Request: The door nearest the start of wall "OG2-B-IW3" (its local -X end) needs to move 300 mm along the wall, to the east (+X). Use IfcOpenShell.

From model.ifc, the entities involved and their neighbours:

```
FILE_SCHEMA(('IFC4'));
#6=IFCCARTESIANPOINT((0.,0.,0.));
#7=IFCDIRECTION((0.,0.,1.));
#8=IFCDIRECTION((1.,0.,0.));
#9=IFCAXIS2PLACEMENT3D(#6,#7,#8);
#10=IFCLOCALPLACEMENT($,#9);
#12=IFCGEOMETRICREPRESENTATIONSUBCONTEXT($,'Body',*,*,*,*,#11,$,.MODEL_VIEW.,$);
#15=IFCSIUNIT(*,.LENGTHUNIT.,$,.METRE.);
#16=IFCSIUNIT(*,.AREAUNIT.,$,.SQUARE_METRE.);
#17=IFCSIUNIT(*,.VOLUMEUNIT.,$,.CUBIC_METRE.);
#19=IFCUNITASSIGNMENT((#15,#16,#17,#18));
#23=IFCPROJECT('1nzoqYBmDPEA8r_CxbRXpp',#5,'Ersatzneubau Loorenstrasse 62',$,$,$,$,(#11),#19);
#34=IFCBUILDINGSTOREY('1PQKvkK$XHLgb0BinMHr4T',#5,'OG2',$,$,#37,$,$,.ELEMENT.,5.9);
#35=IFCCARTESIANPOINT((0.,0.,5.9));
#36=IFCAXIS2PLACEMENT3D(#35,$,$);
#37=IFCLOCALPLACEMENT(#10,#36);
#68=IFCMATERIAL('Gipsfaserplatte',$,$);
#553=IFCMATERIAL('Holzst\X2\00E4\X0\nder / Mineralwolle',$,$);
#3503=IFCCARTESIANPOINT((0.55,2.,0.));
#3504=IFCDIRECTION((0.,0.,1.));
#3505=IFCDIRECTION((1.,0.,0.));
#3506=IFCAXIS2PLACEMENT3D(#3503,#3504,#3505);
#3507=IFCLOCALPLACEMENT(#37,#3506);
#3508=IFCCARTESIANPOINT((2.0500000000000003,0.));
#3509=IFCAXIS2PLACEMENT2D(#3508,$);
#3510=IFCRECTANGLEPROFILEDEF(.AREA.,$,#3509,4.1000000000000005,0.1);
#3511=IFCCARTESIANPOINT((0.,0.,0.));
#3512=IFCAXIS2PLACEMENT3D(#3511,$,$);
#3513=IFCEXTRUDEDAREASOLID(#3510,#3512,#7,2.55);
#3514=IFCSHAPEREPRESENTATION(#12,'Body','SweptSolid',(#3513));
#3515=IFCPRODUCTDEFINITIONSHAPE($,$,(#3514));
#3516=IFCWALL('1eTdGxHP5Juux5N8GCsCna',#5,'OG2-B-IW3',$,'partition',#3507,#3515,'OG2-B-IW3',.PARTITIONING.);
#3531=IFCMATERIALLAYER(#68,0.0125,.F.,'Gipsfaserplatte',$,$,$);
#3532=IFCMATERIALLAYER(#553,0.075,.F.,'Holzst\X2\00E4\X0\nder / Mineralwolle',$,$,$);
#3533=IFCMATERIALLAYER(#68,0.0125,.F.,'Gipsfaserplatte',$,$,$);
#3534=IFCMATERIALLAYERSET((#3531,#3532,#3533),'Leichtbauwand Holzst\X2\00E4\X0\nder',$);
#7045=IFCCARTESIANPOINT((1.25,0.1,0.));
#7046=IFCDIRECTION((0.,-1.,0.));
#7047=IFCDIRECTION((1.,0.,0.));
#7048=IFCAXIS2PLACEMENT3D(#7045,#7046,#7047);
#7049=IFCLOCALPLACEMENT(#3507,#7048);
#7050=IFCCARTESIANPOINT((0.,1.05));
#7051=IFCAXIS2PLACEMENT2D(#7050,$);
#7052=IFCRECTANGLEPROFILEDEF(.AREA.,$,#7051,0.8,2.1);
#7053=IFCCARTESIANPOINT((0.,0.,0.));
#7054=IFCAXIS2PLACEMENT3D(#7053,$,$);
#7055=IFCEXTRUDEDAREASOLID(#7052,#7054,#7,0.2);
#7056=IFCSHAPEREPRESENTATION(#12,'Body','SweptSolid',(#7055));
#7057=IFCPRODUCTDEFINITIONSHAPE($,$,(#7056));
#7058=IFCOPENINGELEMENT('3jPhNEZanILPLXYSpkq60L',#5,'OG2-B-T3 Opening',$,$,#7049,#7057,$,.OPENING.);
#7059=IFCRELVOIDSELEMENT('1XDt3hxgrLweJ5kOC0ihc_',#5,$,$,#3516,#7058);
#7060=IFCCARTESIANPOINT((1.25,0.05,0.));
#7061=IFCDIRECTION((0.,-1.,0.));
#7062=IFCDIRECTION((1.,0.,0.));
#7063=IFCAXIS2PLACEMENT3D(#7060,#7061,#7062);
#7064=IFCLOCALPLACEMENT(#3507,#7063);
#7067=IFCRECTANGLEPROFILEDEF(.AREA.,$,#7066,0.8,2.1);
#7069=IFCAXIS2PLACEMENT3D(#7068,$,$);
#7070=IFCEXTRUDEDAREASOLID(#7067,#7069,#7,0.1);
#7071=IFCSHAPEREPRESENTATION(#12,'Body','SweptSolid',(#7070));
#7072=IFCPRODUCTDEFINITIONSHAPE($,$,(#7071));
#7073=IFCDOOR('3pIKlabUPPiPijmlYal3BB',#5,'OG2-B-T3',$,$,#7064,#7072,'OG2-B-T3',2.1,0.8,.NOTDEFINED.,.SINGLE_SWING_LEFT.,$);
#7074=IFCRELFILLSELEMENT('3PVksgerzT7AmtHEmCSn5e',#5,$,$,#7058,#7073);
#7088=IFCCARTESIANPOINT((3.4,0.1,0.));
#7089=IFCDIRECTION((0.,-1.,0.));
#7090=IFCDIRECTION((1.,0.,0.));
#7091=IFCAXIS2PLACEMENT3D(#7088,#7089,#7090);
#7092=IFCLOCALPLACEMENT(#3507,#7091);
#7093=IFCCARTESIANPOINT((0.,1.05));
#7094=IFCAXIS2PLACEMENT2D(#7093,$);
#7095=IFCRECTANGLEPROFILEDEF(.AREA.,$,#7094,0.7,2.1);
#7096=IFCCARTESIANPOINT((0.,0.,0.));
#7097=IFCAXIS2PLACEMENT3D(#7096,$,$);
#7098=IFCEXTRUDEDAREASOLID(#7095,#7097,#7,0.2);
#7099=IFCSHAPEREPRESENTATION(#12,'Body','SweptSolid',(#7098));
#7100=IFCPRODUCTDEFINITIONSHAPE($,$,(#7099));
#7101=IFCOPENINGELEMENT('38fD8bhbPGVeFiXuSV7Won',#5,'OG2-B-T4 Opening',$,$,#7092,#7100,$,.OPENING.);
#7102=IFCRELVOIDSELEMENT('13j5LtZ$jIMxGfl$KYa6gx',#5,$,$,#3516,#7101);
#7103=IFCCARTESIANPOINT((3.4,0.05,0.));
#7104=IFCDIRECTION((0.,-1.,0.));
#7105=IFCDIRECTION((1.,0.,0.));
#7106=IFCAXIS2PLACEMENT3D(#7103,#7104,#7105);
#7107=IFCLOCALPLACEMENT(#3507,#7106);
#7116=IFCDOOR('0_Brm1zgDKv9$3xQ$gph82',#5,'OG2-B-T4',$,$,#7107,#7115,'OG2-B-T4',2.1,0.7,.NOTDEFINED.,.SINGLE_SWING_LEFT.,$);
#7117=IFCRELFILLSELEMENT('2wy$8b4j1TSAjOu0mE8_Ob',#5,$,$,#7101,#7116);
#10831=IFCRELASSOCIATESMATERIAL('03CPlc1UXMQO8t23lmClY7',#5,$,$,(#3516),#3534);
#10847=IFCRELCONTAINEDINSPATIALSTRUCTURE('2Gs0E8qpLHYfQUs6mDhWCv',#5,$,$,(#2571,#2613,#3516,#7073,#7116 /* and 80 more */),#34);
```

```python
import ifcopenshell
import ifcopenshell.api.geometry
import ifcopenshell.util.placement

model = ifcopenshell.open("model.ifc")

door = model.by_guid("3pIKlabUPPiPijmlYal3BB")
opening = door.FillsVoids[0].RelatingOpeningElement
wall = opening.VoidsElements[0].RelatingBuildingElement

wall_matrix = ifcopenshell.util.placement.get_local_placement(wall.ObjectPlacement)
shift = wall_matrix[:3, 0] * 0.3
before = ifcopenshell.util.placement.get_local_placement(door.ObjectPlacement)[:3, 3].copy()

# The door is not placed relative to its opening, so move both.
for product in (opening, door):
    matrix = ifcopenshell.util.placement.get_local_placement(product.ObjectPlacement)
    matrix[:3, 3] += shift
    ifcopenshell.api.geometry.edit_object_placement(model, product=product, matrix=matrix, is_si=False)

after = ifcopenshell.util.placement.get_local_placement(door.ObjectPlacement)[:3, 3]
print("door moved by", (after - before).round(3) + 0.0)

model.write("model_rev.ifc")
```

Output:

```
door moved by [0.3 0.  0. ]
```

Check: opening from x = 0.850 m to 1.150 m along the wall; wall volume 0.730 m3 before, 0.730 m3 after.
